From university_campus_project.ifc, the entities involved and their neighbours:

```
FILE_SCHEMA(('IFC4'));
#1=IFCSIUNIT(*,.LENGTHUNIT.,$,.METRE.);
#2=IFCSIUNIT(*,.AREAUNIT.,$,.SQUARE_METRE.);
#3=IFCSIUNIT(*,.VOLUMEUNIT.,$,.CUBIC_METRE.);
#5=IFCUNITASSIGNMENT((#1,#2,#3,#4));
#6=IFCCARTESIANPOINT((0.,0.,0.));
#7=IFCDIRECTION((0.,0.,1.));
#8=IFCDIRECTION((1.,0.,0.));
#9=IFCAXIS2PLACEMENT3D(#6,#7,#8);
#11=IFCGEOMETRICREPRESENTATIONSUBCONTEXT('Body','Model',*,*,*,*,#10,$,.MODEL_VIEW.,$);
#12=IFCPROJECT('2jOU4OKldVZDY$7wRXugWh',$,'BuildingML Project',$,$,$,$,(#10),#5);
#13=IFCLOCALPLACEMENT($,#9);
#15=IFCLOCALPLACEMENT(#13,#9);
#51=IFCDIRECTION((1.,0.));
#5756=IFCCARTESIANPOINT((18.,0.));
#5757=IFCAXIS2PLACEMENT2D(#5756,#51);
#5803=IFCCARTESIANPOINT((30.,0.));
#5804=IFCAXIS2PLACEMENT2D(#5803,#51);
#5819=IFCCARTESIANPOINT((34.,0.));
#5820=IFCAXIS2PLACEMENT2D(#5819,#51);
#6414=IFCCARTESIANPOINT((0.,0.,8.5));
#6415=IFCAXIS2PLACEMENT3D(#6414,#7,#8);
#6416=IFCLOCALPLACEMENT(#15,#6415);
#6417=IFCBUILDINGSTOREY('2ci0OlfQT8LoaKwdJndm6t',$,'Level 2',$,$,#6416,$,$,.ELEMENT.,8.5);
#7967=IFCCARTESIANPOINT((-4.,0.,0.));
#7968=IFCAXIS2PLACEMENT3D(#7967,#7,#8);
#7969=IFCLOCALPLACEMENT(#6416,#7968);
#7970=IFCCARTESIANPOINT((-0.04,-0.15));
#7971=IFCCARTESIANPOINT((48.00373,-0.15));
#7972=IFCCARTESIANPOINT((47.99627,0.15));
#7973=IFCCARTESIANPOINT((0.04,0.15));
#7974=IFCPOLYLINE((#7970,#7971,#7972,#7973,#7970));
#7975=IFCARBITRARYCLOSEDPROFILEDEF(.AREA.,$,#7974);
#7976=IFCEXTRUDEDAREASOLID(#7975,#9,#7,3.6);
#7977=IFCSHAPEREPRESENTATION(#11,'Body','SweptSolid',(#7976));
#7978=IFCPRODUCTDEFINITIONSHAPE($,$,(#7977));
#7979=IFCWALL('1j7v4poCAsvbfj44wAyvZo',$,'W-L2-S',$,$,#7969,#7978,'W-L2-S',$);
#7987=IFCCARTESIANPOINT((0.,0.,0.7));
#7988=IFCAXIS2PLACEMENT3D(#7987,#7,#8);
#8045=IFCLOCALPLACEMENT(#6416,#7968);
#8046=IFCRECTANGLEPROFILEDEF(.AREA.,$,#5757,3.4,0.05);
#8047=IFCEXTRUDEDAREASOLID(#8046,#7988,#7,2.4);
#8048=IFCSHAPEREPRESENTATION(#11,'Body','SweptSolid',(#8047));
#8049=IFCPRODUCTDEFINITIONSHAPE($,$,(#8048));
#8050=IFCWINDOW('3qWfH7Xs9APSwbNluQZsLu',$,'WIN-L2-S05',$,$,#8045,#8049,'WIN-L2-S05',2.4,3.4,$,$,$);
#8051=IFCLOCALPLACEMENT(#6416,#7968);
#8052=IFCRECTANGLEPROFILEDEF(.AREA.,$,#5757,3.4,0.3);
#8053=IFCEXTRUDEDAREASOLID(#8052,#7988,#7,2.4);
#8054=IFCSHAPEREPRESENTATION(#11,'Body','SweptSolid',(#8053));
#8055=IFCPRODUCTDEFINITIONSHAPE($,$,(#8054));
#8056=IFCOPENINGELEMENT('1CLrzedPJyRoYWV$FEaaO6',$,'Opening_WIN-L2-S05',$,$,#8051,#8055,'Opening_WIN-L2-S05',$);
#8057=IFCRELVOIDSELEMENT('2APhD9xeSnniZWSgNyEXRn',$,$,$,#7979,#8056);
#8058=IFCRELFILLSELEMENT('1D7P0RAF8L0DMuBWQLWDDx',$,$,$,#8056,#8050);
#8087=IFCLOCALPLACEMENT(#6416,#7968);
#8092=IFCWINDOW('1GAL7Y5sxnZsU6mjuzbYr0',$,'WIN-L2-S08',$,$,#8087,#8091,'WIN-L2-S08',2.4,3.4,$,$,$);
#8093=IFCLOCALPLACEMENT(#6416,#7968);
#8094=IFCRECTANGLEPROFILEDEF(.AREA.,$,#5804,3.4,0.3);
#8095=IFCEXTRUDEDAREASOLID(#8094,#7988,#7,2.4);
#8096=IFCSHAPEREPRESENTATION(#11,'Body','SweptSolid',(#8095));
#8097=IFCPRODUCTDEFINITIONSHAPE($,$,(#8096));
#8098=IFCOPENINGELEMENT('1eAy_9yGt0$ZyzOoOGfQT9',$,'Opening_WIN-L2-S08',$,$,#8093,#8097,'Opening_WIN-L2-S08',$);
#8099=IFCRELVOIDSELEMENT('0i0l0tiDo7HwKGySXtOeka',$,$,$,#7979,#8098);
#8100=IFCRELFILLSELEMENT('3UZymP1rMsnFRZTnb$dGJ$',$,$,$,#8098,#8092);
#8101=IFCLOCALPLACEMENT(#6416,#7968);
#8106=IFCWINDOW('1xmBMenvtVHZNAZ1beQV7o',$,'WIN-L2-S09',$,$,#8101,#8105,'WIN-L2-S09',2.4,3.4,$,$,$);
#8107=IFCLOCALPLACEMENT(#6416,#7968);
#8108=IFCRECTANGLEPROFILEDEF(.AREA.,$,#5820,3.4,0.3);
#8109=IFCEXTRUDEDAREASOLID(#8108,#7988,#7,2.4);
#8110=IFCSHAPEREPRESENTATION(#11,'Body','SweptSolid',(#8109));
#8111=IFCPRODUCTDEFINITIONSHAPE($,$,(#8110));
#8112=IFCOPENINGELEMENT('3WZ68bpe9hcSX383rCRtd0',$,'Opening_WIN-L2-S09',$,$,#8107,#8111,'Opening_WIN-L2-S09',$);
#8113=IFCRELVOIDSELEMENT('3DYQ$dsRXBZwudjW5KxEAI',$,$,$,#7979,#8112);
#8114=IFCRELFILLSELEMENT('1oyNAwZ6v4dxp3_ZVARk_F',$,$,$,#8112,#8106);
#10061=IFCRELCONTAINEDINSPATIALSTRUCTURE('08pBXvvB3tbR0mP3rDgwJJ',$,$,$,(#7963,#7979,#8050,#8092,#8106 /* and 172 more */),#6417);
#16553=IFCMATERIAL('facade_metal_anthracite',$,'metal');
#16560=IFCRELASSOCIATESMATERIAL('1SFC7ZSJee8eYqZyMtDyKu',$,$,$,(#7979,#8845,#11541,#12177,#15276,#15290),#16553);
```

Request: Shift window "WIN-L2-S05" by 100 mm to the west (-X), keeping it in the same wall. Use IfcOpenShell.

```python
import ifcopenshell
import ifcopenshell.api.geometry
import ifcopenshell.util.placement
import ifcopenshell.util.unit

model = ifcopenshell.open("university_campus_project.ifc")
unit_scale = ifcopenshell.util.unit.calculate_unit_scale(model)

window = model.by_id(8050)
opening = window.FillsVoids[0].RelatingOpeningElement
wall = opening.VoidsElements[0].RelatingBuildingElement

wall_matrix = ifcopenshell.util.placement.get_local_placement(wall.ObjectPlacement)
shift = wall_matrix[:3, 0] * -0.1 / unit_scale
before = ifcopenshell.util.placement.get_local_placement(window.ObjectPlacement)[:3, 3].copy()

# The window is not placed relative to its opening, so move both.
for product in (opening, window):
    matrix = ifcopenshell.util.placement.get_local_placement(product.ObjectPlacement)
    matrix[:3, 3] += shift
    ifcopenshell.api.geometry.edit_object_placement(model, product=product, matrix=matrix, is_si=False)

after = ifcopenshell.util.placement.get_local_placement(window.ObjectPlacement)[:3, 3]
print("window moved by", (after - before).round(3) + 0.0)

model.write("university_campus_project-out.ifc")
```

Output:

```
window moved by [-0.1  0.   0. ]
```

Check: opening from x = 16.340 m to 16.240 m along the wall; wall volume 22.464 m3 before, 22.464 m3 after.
